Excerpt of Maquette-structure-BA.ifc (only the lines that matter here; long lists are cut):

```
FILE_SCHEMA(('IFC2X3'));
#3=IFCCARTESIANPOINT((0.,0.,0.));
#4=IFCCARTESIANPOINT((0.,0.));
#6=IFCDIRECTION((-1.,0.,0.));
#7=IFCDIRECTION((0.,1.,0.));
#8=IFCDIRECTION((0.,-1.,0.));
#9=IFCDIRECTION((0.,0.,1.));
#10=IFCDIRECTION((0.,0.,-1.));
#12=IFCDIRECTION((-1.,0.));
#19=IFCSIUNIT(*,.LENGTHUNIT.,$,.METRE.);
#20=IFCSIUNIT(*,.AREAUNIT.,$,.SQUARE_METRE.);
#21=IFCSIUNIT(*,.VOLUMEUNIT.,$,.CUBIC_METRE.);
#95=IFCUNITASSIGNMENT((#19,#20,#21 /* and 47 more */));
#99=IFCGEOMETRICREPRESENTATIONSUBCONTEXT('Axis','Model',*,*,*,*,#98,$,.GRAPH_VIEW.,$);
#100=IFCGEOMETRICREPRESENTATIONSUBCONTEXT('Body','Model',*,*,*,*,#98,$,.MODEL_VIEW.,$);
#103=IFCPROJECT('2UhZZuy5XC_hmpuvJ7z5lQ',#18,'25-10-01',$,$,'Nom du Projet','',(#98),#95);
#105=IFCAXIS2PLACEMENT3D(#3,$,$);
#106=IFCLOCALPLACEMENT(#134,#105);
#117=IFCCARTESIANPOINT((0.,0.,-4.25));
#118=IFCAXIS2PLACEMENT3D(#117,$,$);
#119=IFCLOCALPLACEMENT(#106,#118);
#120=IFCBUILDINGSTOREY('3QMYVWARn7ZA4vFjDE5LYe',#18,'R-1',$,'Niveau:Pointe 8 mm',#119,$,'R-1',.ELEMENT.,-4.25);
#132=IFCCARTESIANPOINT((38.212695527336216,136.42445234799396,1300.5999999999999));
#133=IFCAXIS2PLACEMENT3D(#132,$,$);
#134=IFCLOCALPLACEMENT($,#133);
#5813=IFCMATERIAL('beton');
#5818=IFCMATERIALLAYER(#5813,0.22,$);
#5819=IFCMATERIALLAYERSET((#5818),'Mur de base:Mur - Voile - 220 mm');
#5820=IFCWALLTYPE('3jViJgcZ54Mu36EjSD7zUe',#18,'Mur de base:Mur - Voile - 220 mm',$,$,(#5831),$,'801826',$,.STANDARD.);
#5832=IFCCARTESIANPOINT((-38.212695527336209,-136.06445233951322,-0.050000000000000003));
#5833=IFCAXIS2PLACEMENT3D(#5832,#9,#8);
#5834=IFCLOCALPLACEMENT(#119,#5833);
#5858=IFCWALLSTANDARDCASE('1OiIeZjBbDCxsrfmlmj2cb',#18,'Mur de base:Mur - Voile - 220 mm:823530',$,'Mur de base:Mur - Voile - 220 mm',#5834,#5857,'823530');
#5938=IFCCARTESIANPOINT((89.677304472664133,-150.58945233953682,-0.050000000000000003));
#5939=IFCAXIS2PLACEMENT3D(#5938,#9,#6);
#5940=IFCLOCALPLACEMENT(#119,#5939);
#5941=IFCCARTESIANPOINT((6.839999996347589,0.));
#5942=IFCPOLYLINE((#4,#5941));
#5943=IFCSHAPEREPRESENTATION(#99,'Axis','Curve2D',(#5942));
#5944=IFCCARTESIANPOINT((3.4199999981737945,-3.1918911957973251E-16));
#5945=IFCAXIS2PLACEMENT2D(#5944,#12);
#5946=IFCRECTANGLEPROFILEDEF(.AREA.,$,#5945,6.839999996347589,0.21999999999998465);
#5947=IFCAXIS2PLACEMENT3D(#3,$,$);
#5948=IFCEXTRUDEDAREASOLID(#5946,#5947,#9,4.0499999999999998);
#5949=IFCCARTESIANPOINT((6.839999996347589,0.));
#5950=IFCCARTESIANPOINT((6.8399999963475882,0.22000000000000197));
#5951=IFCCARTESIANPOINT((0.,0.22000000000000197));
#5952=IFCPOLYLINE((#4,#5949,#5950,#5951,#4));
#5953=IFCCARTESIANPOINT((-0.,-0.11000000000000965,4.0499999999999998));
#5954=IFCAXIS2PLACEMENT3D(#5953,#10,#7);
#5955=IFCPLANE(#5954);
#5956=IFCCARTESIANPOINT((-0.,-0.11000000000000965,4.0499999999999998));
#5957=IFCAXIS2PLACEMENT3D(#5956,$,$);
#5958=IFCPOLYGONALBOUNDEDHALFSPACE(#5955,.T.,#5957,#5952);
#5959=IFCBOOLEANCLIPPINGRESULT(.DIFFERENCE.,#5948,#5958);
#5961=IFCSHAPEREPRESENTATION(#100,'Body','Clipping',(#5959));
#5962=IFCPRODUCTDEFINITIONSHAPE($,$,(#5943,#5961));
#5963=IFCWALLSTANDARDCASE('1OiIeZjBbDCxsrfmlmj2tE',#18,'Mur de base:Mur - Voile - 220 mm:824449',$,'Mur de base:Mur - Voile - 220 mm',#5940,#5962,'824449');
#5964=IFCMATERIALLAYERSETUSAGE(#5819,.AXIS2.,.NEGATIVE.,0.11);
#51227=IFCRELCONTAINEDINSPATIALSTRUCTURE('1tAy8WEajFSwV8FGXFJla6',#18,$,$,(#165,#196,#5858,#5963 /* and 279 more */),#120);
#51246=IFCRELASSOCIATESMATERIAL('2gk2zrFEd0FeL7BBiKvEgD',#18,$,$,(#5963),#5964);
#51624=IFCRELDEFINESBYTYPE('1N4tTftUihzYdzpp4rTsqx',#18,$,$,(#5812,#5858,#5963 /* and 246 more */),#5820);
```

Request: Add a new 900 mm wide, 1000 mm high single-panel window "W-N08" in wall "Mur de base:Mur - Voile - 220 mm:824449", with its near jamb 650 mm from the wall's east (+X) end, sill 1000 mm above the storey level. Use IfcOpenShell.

```python
import numpy as np
import ifcopenshell
import ifcopenshell.api.feature
import ifcopenshell.api.geometry
import ifcopenshell.api.root
import ifcopenshell.api.spatial
import ifcopenshell.api.type
import ifcopenshell.geom
import ifcopenshell.util.element
import ifcopenshell.util.placement
import ifcopenshell.util.representation
import ifcopenshell.util.shape
import ifcopenshell.util.unit

model = ifcopenshell.open("Maquette-structure-BA.ifc")
unit_scale = ifcopenshell.util.unit.calculate_unit_scale(model)
settings = ifcopenshell.geom.settings()


def volume(element):
    """Net volume in cubic metres, openings subtracted."""
    shape = ifcopenshell.geom.create_shape(settings, element)
    return ifcopenshell.util.shape.get_volume(shape.geometry)


wall = model.by_id(5963)
storey = ifcopenshell.util.element.get_container(wall, ifc_class="IfcBuildingStorey")
context = ifcopenshell.util.representation.get_context(model, "Model", "Body", "MODEL_VIEW")
before = volume(wall)

width, height, from_end, sill = 0.9, 1, 0.65, 1  # metres

# The wall runs along its own X axis, and the end named is its -X end.
wall_shape = ifcopenshell.geom.create_shape(settings, wall)
x, y, z = ifcopenshell.util.shape.get_vertices(wall_shape.geometry).T
start = x.min() + from_end
face, thickness = float(y.min()), float(y.max() - y.min())
wall_matrix = ifcopenshell.util.placement.get_local_placement(wall.ObjectPlacement)
level = ifcopenshell.util.placement.get_local_placement(storey.ObjectPlacement)[2, 3]


def in_wall(x, y):
    """Placement at x, y metres in the wall's axes, at sill height."""
    matrix = wall_matrix.copy()
    matrix[:, 3] = wall_matrix @ np.array([x / unit_scale, y / unit_scale, 0.0, 1.0])
    matrix[2, 3] = level + sill / unit_scale
    return matrix


# Opening: a box that overshoots both wall faces by 50 mm.
opening = ifcopenshell.api.root.create_entity(model, ifc_class="IfcOpeningElement")
box = ifcopenshell.api.geometry.add_wall_representation(
    model, context=context, length=width, height=height, thickness=thickness + 0.1
)
ifcopenshell.api.geometry.assign_representation(model, product=opening, representation=box)
ifcopenshell.api.geometry.edit_object_placement(model, product=opening, matrix=in_wall(start, face - 0.05), is_si=False)
ifcopenshell.api.feature.add_feature(model, feature=opening, element=wall)

window = ifcopenshell.api.root.create_entity(model, ifc_class="IfcWindow", name="W-N08")
window.OverallWidth, window.OverallHeight = width / unit_scale, height / unit_scale
body = ifcopenshell.api.geometry.add_window_representation(
    model,
    context=context,
    overall_width=window.OverallWidth,
    overall_height=window.OverallHeight,
    partition_type="SINGLE_PANEL",
)
ifcopenshell.api.geometry.assign_representation(model, product=window, representation=body)
ifcopenshell.api.spatial.assign_container(model, products=[window], relating_structure=storey)
fills = ifcopenshell.api.feature.add_filling(model, opening=opening, element=window)
fills.OwnerHistory = window.OwnerHistory  # required in IFC2X3

# IFC2X3 keeps the operation on the window style.
style = ifcopenshell.api.root.create_entity(model, ifc_class="IfcWindowStyle", name="W-N08")
style.OperationType, style.ConstructionType = "SINGLE_PANEL", "NOTDEFINED"
style.ParameterTakesPrecedence = style.Sizeable = False
ifcopenshell.api.type.assign_type(model, related_objects=[window], relating_type=style)

# Centre the window in the wall's thickness.
ifcopenshell.api.geometry.edit_object_placement(model, product=window, matrix=in_wall(start, face), is_si=False)
window_shape = ifcopenshell.geom.create_shape(settings, window)
depth = ifcopenshell.util.shape.get_vertices(window_shape.geometry)[:, 1]
offset = face + thickness / 2 - (depth.min() + depth.max()) / 2
ifcopenshell.api.geometry.edit_object_placement(model, product=window, matrix=in_wall(start, offset), is_si=False)

after = volume(wall)

print(f"wall volume {before:.3f} -> {after:.3f} m3")

model.write("Maquette-structure-BA-out.ifc")
```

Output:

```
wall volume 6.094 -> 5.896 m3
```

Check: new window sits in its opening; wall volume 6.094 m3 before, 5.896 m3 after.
